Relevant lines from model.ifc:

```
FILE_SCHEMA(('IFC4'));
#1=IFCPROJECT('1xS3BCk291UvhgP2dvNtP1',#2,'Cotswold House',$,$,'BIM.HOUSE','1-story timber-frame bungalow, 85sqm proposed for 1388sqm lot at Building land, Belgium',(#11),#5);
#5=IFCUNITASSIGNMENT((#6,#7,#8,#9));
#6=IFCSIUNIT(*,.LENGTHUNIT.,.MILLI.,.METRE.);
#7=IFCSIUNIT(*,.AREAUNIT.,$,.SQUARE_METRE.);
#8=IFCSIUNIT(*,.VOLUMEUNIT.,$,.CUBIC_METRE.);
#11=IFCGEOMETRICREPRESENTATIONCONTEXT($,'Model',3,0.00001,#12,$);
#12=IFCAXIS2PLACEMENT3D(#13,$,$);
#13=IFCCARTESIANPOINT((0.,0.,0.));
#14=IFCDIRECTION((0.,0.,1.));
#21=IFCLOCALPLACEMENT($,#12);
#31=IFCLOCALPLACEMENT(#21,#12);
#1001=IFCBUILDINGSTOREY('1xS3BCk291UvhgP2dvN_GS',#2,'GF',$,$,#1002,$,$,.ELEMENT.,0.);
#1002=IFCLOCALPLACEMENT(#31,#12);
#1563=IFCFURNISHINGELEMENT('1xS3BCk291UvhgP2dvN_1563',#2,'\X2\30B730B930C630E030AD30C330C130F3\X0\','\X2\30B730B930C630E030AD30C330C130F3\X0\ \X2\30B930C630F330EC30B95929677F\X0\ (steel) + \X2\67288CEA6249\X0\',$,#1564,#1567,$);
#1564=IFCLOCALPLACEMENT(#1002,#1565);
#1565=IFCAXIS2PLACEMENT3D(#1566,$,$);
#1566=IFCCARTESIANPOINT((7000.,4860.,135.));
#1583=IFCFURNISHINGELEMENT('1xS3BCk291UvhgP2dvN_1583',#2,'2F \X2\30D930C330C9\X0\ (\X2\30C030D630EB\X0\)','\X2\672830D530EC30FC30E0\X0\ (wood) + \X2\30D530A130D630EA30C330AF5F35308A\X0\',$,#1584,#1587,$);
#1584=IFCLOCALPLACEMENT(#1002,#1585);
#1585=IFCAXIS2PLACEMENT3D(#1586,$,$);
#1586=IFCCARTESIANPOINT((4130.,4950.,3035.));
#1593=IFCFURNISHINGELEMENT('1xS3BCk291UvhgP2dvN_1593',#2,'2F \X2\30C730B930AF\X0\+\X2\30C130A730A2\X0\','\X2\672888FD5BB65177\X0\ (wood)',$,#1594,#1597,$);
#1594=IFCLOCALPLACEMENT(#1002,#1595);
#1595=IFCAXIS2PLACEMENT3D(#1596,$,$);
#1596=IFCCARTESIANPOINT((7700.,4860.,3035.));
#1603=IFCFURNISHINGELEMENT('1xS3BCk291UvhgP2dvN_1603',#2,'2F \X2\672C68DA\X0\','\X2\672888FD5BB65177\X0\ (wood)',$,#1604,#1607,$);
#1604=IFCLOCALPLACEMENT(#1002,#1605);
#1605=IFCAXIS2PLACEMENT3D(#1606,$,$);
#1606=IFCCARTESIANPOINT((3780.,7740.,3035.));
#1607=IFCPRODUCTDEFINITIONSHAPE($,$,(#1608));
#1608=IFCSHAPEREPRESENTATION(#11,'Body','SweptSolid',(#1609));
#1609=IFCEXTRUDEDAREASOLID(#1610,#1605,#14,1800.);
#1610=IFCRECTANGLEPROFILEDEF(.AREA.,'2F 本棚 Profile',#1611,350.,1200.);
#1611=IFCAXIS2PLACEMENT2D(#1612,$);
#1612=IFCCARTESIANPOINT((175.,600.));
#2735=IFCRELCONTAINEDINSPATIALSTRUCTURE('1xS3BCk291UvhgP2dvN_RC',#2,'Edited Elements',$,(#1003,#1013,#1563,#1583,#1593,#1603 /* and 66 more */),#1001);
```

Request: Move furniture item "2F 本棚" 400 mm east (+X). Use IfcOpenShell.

```python
import ifcopenshell
import ifcopenshell.api.geometry
import ifcopenshell.util.placement

model = ifcopenshell.open("model.ifc")

item = model.by_id(1603)
matrix = ifcopenshell.util.placement.get_local_placement(item.ObjectPlacement)
matrix[0, 3] += 400.0
ifcopenshell.api.geometry.edit_object_placement(model, product=item, matrix=matrix, is_si=False)

print(ifcopenshell.util.placement.get_local_placement(item.ObjectPlacement).round(3) + 0.0)

model.write("model_updated.ifc")
```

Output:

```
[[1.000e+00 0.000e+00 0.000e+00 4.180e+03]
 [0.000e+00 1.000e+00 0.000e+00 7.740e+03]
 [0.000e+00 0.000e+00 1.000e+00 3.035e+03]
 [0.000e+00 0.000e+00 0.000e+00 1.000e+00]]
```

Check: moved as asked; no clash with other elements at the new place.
